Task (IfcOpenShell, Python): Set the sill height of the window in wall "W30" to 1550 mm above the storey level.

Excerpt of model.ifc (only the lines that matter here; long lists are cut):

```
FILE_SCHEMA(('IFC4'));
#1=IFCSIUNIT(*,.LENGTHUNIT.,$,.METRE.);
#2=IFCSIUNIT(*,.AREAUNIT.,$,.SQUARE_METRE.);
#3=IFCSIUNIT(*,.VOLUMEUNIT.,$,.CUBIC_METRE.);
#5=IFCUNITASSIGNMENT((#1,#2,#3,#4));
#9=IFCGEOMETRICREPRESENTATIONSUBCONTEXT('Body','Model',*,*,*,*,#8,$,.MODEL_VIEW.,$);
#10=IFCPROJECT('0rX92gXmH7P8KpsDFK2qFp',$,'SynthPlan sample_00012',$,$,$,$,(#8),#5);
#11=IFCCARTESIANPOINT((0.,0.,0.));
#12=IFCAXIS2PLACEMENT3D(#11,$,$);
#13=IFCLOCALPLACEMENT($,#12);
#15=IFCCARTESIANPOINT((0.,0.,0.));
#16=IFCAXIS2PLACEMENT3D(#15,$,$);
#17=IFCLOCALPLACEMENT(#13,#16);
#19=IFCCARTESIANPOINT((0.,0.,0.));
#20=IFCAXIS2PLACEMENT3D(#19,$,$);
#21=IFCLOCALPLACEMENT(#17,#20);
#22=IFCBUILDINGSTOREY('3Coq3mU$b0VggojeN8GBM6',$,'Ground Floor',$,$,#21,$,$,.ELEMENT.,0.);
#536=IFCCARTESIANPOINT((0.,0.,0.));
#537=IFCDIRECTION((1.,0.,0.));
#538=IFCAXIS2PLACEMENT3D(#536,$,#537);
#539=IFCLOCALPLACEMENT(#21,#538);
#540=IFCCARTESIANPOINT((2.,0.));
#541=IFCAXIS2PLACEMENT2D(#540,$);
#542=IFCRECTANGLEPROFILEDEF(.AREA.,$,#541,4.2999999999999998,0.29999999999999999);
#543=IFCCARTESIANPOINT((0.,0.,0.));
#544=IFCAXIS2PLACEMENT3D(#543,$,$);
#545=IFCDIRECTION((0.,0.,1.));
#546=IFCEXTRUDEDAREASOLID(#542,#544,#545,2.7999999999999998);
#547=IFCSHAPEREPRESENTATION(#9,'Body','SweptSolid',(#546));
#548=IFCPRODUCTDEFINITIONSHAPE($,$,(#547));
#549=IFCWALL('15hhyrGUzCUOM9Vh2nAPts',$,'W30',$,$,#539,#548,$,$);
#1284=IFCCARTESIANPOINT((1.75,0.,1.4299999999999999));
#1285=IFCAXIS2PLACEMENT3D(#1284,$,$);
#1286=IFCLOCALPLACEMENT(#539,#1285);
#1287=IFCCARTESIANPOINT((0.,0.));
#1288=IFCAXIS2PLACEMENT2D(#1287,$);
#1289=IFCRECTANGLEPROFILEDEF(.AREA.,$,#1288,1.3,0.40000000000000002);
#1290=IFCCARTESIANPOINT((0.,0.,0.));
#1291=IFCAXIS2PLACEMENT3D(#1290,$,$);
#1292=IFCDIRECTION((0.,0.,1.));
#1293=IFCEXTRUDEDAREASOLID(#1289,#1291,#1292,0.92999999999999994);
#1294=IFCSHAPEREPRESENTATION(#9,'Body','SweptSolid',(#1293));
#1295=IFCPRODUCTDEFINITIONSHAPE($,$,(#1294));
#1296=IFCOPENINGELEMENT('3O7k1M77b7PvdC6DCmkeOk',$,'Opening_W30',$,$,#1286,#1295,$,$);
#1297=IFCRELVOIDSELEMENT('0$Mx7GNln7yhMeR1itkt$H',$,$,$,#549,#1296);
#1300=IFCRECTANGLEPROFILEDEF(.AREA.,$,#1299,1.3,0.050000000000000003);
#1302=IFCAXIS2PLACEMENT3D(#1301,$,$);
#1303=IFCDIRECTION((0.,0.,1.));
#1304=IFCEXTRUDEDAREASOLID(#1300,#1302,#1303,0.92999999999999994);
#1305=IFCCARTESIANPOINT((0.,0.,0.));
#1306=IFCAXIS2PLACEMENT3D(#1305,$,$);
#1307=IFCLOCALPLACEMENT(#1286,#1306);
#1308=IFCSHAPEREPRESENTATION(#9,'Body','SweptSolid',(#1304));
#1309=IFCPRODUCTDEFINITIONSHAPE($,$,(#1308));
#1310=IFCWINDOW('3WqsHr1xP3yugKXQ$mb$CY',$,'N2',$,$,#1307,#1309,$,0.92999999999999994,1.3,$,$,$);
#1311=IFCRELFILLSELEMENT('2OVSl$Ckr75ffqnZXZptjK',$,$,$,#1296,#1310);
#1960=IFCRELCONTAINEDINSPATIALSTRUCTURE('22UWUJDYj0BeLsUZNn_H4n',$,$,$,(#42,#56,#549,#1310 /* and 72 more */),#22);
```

```python
import numpy as np
import ifcopenshell
import ifcopenshell.api.geometry
import ifcopenshell.geom
import ifcopenshell.util.element
import ifcopenshell.util.placement
import ifcopenshell.util.shape
import ifcopenshell.util.unit

model = ifcopenshell.open("model.ifc")
unit_scale = ifcopenshell.util.unit.calculate_unit_scale(model)

window = model.by_guid("3WqsHr1xP3yugKXQ$mb$CY")
opening = window.FillsVoids[0].RelatingOpeningElement
storey = ifcopenshell.util.element.get_container(window, ifc_class="IfcBuildingStorey")
level = ifcopenshell.util.placement.get_local_placement(storey.ObjectPlacement)[2, 3]

# The opening's origin need not be at the sill, so measure its lowest point.
shape = ifcopenshell.geom.create_shape(ifcopenshell.geom.settings(), opening)
bottom = ifcopenshell.util.shape.get_shape_bottom_elevation(shape, shape.geometry) / unit_scale
dz = level + 1.55 / unit_scale - bottom

shift = np.array([0.0, 0.0, dz])
# The window is placed relative to its opening, so it follows when the opening moves.
matrix = ifcopenshell.util.placement.get_local_placement(opening.ObjectPlacement)
matrix[:3, 3] += shift
ifcopenshell.api.geometry.edit_object_placement(
    model, product=opening, matrix=matrix, is_si=False, should_transform_children=True
)

print(f"moved by {dz * unit_scale:+.3f} m")

model.write("model_rev.ifc")
```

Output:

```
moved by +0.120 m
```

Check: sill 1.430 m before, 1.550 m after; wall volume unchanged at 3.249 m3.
